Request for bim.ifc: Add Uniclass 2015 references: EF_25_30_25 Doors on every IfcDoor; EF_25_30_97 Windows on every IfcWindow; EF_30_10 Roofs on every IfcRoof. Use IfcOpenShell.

First a look at what the model holds.

```python
import ifcopenshell

model = ifcopenshell.open("bim.ifc")
print(model.schema)
print("classifications:", [c.Name for c in model.by_type("IfcClassification")])
for ifc_class in ("IfcDoor", "IfcRoof", "IfcStair", "IfcWall", "IfcWindow"):
    print(ifc_class, len(model.by_type(ifc_class)))
```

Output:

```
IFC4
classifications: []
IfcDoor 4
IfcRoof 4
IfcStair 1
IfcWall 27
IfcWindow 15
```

```python
import ifcopenshell
import ifcopenshell.api.classification

model = ifcopenshell.open("bim.ifc")

system = ifcopenshell.api.classification.add_classification(model, classification="Uniclass 2015")

codes = {
    "IfcDoor": ("EF_25_30_25", "Doors"),
    "IfcWindow": ("EF_25_30_97", "Windows"),
    "IfcRoof": ("EF_30_10", "Roofs"),
}
for ifc_class, (code, name) in codes.items():
    products = model.by_type(ifc_class)
    ifcopenshell.api.classification.add_reference(
        model, products=products, classification=system, identification=code, name=name
    )
    print(code, len(products))

model.write("bim_updated.ifc")
```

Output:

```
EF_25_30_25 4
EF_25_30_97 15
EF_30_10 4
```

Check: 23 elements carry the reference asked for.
